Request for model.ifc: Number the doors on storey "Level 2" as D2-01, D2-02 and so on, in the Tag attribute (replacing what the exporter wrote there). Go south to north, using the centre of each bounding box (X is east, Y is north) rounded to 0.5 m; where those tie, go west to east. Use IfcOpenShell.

First a look at what the model holds.

```python
import ifcopenshell
import ifcopenshell.util.element
import ifcopenshell.util.placement

model = ifcopenshell.open("model.ifc")
print(model.schema)
storey = next(s for s in model.by_type("IfcBuildingStorey") if s.Name == "Level 2")
doors = [e for e in ifcopenshell.util.element.get_decomposition(storey) if e.is_a("IfcDoor")]
for e in sorted(doors, key=lambda e: e.id()):
    origin = ifcopenshell.util.placement.get_local_placement(e.ObjectPlacement)[:3, 3]
    print(e.id(), e.Tag, e.Name, origin.round(2) + 0.0, sep=" | ")
```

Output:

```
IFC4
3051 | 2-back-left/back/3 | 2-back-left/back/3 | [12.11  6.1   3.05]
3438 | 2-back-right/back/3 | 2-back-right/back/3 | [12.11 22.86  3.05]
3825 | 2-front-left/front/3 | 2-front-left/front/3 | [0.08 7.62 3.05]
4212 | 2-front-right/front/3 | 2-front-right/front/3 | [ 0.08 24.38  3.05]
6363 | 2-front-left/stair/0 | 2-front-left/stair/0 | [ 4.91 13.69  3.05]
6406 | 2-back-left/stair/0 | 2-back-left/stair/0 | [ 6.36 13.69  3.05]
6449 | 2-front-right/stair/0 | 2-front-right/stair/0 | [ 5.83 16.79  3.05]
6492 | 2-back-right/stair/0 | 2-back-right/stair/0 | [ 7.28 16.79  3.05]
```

```python
import ifcopenshell
import ifcopenshell.geom
import ifcopenshell.util.element
import ifcopenshell.util.shape

model = ifcopenshell.open("model.ifc")
settings = ifcopenshell.geom.settings()
settings.set("use-world-coords", True)


def centre(element):
    shape = ifcopenshell.geom.create_shape(settings, element)
    return ifcopenshell.util.shape.get_bbox_centroid(shape.geometry)


storey = next(s for s in model.by_type("IfcBuildingStorey") if s.Name == "Level 2")
doors = [e for e in ifcopenshell.util.element.get_decomposition(storey) if e.is_a("IfcDoor")]

# Insertion points can sit at a corner or the storey origin, so sort by the geometry (in metres).
centres = {e: centre(e) for e in doors}
doors.sort(key=lambda e: (round(centres[e][1] / 0.5), centres[e][0]))

for i, e in enumerate(doors, start=1):
    number = f"D2-{i:02d}"
    e.Tag = number
    print(e.id(), number)

model.write("model_v2.ifc")
```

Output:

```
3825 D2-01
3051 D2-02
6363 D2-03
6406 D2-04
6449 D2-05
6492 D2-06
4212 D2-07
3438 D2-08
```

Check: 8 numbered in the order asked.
